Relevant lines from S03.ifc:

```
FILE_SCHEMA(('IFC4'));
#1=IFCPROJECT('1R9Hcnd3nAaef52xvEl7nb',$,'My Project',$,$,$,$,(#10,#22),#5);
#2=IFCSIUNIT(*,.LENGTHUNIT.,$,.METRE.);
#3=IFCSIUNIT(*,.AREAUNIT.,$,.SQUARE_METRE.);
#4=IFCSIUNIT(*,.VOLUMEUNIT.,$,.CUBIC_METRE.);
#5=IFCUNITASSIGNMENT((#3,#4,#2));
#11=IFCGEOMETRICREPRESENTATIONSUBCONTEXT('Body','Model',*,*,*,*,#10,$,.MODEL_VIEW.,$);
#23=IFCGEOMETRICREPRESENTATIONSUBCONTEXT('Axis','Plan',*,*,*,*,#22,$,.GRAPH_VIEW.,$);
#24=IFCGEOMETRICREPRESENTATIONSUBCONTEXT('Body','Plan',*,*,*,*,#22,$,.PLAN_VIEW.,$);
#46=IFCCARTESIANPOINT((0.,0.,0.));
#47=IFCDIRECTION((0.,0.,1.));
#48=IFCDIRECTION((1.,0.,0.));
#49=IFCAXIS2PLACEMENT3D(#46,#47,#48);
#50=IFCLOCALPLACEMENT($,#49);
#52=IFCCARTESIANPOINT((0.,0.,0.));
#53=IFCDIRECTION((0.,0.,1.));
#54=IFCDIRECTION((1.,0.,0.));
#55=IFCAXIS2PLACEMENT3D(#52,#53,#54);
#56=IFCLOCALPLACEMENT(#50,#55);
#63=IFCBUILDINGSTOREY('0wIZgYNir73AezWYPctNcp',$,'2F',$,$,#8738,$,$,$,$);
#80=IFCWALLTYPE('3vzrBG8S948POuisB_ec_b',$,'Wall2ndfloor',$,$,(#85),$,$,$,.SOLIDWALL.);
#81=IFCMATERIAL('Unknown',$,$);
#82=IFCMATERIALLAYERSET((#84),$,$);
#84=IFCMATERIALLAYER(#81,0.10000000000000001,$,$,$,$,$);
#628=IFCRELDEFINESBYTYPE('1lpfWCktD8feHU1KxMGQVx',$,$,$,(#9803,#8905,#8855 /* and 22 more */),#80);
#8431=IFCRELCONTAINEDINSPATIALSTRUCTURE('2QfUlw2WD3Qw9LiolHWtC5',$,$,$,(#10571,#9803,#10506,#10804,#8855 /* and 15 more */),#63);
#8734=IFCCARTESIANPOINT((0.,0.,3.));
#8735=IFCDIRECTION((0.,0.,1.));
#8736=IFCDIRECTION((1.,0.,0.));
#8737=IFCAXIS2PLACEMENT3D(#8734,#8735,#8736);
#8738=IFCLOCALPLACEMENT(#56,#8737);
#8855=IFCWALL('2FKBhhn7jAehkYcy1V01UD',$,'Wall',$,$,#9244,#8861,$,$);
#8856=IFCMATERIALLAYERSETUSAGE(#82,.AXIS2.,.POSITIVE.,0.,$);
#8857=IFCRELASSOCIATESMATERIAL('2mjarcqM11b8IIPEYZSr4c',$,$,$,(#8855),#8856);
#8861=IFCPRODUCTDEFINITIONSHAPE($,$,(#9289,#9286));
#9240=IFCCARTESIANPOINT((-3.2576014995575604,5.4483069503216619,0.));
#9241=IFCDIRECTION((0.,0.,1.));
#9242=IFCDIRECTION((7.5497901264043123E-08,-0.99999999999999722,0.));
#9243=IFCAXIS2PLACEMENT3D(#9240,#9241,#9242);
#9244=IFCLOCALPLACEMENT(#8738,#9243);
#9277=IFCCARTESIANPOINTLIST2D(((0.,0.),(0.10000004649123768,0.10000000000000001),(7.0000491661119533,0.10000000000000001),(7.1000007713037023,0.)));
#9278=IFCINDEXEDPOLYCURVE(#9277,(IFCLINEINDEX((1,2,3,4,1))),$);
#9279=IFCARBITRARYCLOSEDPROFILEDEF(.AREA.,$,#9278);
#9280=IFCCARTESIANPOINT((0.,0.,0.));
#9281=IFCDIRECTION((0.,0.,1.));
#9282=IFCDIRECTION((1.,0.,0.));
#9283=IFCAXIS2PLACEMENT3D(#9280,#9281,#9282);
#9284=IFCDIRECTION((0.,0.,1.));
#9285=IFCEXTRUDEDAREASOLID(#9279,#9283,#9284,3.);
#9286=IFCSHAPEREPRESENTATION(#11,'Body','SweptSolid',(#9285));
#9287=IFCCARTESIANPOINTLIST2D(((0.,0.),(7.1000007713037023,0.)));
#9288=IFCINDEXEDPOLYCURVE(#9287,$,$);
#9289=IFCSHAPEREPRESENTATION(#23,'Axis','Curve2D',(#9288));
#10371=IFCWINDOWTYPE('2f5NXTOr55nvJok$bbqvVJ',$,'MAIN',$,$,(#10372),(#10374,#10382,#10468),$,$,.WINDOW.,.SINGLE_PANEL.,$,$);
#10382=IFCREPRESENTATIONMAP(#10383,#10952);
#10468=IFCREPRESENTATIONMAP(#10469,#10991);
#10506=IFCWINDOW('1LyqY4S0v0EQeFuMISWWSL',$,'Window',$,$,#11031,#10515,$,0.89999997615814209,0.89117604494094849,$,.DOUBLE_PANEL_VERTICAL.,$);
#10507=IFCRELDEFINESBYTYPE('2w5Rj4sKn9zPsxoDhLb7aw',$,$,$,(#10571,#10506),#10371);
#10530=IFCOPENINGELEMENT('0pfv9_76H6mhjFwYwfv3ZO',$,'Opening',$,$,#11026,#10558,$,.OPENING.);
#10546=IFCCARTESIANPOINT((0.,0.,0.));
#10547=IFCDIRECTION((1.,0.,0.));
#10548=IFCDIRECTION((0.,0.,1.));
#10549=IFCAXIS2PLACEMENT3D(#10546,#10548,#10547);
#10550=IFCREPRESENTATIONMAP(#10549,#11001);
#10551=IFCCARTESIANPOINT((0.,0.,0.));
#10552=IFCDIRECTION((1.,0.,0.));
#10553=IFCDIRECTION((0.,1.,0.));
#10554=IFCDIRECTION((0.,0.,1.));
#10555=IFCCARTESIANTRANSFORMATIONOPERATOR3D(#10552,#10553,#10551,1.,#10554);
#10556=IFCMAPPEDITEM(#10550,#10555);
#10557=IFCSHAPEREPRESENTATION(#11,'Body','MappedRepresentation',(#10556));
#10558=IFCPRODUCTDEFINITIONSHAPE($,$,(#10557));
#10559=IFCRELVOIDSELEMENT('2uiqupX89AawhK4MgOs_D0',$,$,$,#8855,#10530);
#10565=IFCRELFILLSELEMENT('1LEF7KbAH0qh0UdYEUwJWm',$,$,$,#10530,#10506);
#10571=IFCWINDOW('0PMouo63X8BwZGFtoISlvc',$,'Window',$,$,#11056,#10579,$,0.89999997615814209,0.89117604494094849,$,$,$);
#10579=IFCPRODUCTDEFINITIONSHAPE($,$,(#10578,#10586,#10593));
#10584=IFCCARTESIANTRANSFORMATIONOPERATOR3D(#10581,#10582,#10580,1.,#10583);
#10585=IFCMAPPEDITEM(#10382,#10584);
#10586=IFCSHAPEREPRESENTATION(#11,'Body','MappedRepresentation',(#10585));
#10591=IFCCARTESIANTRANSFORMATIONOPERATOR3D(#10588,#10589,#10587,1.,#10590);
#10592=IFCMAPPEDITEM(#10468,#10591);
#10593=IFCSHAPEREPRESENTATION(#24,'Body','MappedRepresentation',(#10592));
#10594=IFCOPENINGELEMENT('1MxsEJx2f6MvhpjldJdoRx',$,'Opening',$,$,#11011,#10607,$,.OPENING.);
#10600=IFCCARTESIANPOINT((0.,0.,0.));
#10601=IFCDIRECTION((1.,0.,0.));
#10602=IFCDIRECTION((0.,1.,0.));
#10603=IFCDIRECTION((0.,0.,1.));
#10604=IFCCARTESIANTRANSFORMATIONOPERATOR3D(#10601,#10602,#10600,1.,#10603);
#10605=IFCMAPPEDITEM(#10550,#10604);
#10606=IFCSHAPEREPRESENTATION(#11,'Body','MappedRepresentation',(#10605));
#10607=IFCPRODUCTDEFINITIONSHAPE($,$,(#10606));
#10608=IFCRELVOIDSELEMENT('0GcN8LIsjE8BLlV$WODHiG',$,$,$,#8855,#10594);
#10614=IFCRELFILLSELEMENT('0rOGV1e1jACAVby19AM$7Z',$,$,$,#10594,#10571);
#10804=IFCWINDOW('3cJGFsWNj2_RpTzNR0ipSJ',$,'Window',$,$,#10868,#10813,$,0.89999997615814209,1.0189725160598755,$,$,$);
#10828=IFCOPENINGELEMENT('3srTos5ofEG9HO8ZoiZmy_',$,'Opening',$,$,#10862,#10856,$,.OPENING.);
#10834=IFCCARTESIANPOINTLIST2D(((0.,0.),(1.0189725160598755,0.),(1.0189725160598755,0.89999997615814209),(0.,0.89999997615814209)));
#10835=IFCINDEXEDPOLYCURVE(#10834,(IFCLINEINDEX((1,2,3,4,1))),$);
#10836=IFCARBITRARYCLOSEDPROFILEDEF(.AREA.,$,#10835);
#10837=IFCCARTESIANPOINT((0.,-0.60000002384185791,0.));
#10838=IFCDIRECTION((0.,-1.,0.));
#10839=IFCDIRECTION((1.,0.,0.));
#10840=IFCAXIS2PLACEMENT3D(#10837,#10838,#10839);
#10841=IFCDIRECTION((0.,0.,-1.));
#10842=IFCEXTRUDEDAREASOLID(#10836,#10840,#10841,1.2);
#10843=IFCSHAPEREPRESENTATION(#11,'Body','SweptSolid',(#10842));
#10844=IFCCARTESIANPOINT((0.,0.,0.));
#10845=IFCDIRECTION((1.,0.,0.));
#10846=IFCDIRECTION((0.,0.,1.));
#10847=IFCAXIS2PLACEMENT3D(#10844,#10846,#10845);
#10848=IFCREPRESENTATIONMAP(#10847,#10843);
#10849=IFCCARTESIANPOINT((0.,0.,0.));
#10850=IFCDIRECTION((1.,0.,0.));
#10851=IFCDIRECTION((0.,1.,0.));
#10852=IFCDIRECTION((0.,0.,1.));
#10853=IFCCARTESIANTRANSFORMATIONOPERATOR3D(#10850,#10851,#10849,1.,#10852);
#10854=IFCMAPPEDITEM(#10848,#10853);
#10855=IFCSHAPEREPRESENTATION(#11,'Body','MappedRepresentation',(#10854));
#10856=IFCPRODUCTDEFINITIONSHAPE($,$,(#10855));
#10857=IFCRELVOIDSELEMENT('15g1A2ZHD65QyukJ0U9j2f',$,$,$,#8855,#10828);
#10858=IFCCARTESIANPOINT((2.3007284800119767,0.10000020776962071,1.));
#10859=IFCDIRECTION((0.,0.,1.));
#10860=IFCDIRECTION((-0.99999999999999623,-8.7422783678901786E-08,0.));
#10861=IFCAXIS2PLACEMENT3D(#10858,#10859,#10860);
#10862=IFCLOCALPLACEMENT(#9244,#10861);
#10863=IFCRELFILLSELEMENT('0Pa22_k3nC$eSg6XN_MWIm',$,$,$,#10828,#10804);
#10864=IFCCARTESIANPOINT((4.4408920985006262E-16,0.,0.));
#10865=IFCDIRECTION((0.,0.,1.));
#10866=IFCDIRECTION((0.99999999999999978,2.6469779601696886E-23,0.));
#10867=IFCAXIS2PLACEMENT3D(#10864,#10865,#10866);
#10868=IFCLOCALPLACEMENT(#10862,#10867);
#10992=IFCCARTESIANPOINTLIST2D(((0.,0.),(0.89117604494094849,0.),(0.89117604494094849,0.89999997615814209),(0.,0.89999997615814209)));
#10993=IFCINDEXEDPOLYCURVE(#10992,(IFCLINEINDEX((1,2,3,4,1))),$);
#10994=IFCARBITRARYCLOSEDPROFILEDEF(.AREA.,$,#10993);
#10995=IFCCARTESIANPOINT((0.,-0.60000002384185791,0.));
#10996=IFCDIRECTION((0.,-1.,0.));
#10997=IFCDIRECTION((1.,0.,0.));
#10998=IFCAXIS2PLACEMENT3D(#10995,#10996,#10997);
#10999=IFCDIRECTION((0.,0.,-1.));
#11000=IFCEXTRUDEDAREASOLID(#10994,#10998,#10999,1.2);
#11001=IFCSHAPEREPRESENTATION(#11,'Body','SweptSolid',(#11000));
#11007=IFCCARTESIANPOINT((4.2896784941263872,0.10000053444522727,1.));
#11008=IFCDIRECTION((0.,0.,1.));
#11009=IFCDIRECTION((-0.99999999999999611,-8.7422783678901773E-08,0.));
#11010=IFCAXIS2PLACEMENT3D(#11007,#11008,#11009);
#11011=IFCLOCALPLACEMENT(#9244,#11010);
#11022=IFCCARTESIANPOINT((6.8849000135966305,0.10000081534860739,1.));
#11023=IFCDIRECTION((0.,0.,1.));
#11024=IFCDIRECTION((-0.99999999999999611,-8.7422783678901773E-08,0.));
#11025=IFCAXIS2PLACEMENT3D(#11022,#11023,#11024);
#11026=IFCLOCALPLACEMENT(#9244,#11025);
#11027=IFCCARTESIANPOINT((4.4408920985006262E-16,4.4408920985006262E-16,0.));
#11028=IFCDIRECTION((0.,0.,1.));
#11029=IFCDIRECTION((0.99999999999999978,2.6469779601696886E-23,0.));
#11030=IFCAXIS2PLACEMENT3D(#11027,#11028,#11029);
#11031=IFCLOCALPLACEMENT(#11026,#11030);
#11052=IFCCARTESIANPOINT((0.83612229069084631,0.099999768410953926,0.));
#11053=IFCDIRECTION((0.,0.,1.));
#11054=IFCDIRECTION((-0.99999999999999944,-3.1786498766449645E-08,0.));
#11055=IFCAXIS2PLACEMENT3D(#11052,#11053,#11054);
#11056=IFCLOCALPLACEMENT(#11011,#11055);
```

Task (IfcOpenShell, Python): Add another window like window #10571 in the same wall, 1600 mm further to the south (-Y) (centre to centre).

```python
import ifcopenshell
import ifcopenshell.api.feature
import ifcopenshell.api.geometry
import ifcopenshell.api.root
import ifcopenshell.geom
import ifcopenshell.util.element
import ifcopenshell.util.placement
import ifcopenshell.util.shape

model = ifcopenshell.open("S03.ifc")
settings = ifcopenshell.geom.settings()


def volume(element):
    """Net volume in cubic metres, openings subtracted."""
    shape = ifcopenshell.geom.create_shape(settings, element)
    return ifcopenshell.util.shape.get_volume(shape.geometry)


window = model.by_guid("0PMouo63X8BwZGFtoISlvc")
opening = window.FillsVoids[0].RelatingOpeningElement
wall = opening.VoidsElements[0].RelatingBuildingElement
before = volume(wall)
shift = ifcopenshell.util.placement.get_local_placement(wall.ObjectPlacement)[:3, 0] * 1.6

# copy_class copies the void relationship, type, container and properties, but no geometry.
new_opening = ifcopenshell.api.root.copy_class(model, product=opening)
new_opening.Representation = ifcopenshell.util.element.copy_deep(
    model, opening.Representation, exclude=["IfcGeometricRepresentationContext", "IfcRepresentationMap"]
)
new_window = ifcopenshell.api.root.copy_class(model, product=window)
new_window.Representation = ifcopenshell.util.element.copy_deep(
    model, window.Representation, exclude=["IfcGeometricRepresentationContext", "IfcRepresentationMap"]
)
ifcopenshell.api.feature.add_filling(model, opening=new_opening, element=new_window)

for old, new in ((opening, new_opening), (window, new_window)):
    matrix = ifcopenshell.util.placement.get_local_placement(old.ObjectPlacement)
    matrix[:3, 3] += shift
    ifcopenshell.api.geometry.edit_object_placement(model, product=new, matrix=matrix, is_si=False)

after = volume(wall)

print(f"wall volume {before:.3f} -> {after:.3f} m3")

model.write("S03-out.ifc")
```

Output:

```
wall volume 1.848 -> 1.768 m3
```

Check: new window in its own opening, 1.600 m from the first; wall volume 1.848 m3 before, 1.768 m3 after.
